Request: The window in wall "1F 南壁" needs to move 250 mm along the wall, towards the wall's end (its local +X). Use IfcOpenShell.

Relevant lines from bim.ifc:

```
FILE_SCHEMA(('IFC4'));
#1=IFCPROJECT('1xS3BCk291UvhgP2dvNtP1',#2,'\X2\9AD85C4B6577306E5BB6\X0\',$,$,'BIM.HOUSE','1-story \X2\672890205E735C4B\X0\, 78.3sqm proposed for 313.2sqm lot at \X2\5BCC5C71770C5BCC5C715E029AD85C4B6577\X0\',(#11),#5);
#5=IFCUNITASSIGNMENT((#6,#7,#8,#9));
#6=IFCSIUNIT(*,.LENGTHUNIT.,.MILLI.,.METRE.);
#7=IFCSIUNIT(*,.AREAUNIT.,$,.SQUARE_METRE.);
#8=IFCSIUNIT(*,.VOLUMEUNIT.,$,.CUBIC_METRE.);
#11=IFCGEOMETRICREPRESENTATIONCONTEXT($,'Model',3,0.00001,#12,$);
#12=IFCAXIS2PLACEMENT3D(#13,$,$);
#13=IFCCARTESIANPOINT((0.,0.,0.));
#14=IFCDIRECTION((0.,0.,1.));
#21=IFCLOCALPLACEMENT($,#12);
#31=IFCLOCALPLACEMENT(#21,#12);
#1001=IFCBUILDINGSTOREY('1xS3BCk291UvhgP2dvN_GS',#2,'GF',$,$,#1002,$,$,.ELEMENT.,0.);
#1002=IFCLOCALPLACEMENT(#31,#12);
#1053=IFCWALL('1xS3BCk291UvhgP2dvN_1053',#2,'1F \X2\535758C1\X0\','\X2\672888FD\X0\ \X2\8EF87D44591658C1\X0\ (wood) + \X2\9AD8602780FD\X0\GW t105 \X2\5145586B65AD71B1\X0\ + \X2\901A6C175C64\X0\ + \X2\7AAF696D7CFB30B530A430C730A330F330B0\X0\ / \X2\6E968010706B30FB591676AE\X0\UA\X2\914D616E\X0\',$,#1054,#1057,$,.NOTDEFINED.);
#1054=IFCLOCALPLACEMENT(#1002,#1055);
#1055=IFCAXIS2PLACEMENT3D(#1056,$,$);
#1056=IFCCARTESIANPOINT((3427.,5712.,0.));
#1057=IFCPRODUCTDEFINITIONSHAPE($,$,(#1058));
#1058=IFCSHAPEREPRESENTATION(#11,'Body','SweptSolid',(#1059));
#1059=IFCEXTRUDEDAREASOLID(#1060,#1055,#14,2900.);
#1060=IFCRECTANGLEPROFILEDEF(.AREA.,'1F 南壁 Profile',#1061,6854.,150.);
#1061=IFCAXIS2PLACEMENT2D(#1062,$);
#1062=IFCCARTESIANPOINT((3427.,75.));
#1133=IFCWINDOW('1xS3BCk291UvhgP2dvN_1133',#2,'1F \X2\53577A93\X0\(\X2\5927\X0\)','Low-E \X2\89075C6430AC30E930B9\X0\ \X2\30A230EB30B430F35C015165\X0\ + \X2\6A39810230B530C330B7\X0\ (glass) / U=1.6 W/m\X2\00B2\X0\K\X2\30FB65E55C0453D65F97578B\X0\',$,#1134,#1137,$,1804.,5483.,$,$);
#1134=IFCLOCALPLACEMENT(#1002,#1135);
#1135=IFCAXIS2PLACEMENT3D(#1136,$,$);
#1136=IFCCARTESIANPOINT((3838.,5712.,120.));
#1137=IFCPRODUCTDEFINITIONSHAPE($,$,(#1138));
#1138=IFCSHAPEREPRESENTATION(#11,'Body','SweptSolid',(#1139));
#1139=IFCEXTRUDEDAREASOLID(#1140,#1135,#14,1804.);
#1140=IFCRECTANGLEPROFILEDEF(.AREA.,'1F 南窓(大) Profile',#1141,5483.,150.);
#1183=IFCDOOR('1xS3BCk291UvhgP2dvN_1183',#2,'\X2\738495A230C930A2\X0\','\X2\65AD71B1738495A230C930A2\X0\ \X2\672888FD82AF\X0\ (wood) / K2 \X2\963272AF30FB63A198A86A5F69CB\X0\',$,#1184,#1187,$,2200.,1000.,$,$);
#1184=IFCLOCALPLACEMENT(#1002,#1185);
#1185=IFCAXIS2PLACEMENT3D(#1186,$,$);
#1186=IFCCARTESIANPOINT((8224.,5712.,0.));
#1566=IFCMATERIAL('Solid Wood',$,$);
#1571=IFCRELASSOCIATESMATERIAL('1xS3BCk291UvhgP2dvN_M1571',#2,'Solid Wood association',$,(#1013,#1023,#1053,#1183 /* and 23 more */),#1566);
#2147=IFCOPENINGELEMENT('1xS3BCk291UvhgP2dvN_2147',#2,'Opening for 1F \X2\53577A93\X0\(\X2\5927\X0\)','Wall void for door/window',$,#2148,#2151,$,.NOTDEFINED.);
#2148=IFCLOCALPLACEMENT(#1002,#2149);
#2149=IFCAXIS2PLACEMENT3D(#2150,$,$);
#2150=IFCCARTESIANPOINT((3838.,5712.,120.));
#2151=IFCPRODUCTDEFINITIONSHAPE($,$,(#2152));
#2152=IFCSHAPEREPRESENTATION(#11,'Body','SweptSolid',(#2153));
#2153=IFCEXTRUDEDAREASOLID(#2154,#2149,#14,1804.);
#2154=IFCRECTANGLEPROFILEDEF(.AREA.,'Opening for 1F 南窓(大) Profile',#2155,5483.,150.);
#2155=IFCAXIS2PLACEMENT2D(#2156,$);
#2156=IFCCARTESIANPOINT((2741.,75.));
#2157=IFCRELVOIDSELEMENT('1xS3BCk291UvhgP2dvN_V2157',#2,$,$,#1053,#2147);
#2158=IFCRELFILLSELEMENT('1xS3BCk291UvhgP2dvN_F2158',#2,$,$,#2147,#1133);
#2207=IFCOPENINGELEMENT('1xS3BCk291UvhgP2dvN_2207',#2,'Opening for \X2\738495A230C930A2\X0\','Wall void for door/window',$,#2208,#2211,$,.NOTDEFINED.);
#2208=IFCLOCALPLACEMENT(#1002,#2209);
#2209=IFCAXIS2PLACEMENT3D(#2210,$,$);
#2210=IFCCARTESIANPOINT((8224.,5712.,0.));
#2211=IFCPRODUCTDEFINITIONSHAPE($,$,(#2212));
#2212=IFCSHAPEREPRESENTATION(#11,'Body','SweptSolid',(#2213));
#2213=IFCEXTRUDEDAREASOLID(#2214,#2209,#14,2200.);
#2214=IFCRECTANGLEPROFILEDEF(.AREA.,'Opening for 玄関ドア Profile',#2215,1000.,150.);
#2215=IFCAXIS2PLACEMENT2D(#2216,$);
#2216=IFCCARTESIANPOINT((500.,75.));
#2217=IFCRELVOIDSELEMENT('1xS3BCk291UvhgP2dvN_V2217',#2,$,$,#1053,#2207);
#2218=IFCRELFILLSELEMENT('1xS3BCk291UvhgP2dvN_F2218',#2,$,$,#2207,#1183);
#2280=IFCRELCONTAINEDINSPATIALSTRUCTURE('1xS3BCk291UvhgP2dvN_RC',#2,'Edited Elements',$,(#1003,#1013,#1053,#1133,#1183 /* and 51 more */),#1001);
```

```python
import ifcopenshell
import ifcopenshell.api.geometry
import ifcopenshell.util.placement
import ifcopenshell.util.unit

model = ifcopenshell.open("bim.ifc")
unit_scale = ifcopenshell.util.unit.calculate_unit_scale(model)

window = model.by_guid("1xS3BCk291UvhgP2dvN_1133")
opening = window.FillsVoids[0].RelatingOpeningElement
wall = opening.VoidsElements[0].RelatingBuildingElement

wall_matrix = ifcopenshell.util.placement.get_local_placement(wall.ObjectPlacement)
shift = wall_matrix[:3, 0] * 0.25 / unit_scale
before = ifcopenshell.util.placement.get_local_placement(window.ObjectPlacement)[:3, 3].copy()

# The window is not placed relative to its opening, so move both.
for product in (opening, window):
    matrix = ifcopenshell.util.placement.get_local_placement(product.ObjectPlacement)
    matrix[:3, 3] += shift
    ifcopenshell.api.geometry.edit_object_placement(model, product=product, matrix=matrix, is_si=False)

after = ifcopenshell.util.placement.get_local_placement(window.ObjectPlacement)[:3, 3]
print("window moved by", (after - before).round(3) + 0.0)

model.write("bim_updated.ifc")
```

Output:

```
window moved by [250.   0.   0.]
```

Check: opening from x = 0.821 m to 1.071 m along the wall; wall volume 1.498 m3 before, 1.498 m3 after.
